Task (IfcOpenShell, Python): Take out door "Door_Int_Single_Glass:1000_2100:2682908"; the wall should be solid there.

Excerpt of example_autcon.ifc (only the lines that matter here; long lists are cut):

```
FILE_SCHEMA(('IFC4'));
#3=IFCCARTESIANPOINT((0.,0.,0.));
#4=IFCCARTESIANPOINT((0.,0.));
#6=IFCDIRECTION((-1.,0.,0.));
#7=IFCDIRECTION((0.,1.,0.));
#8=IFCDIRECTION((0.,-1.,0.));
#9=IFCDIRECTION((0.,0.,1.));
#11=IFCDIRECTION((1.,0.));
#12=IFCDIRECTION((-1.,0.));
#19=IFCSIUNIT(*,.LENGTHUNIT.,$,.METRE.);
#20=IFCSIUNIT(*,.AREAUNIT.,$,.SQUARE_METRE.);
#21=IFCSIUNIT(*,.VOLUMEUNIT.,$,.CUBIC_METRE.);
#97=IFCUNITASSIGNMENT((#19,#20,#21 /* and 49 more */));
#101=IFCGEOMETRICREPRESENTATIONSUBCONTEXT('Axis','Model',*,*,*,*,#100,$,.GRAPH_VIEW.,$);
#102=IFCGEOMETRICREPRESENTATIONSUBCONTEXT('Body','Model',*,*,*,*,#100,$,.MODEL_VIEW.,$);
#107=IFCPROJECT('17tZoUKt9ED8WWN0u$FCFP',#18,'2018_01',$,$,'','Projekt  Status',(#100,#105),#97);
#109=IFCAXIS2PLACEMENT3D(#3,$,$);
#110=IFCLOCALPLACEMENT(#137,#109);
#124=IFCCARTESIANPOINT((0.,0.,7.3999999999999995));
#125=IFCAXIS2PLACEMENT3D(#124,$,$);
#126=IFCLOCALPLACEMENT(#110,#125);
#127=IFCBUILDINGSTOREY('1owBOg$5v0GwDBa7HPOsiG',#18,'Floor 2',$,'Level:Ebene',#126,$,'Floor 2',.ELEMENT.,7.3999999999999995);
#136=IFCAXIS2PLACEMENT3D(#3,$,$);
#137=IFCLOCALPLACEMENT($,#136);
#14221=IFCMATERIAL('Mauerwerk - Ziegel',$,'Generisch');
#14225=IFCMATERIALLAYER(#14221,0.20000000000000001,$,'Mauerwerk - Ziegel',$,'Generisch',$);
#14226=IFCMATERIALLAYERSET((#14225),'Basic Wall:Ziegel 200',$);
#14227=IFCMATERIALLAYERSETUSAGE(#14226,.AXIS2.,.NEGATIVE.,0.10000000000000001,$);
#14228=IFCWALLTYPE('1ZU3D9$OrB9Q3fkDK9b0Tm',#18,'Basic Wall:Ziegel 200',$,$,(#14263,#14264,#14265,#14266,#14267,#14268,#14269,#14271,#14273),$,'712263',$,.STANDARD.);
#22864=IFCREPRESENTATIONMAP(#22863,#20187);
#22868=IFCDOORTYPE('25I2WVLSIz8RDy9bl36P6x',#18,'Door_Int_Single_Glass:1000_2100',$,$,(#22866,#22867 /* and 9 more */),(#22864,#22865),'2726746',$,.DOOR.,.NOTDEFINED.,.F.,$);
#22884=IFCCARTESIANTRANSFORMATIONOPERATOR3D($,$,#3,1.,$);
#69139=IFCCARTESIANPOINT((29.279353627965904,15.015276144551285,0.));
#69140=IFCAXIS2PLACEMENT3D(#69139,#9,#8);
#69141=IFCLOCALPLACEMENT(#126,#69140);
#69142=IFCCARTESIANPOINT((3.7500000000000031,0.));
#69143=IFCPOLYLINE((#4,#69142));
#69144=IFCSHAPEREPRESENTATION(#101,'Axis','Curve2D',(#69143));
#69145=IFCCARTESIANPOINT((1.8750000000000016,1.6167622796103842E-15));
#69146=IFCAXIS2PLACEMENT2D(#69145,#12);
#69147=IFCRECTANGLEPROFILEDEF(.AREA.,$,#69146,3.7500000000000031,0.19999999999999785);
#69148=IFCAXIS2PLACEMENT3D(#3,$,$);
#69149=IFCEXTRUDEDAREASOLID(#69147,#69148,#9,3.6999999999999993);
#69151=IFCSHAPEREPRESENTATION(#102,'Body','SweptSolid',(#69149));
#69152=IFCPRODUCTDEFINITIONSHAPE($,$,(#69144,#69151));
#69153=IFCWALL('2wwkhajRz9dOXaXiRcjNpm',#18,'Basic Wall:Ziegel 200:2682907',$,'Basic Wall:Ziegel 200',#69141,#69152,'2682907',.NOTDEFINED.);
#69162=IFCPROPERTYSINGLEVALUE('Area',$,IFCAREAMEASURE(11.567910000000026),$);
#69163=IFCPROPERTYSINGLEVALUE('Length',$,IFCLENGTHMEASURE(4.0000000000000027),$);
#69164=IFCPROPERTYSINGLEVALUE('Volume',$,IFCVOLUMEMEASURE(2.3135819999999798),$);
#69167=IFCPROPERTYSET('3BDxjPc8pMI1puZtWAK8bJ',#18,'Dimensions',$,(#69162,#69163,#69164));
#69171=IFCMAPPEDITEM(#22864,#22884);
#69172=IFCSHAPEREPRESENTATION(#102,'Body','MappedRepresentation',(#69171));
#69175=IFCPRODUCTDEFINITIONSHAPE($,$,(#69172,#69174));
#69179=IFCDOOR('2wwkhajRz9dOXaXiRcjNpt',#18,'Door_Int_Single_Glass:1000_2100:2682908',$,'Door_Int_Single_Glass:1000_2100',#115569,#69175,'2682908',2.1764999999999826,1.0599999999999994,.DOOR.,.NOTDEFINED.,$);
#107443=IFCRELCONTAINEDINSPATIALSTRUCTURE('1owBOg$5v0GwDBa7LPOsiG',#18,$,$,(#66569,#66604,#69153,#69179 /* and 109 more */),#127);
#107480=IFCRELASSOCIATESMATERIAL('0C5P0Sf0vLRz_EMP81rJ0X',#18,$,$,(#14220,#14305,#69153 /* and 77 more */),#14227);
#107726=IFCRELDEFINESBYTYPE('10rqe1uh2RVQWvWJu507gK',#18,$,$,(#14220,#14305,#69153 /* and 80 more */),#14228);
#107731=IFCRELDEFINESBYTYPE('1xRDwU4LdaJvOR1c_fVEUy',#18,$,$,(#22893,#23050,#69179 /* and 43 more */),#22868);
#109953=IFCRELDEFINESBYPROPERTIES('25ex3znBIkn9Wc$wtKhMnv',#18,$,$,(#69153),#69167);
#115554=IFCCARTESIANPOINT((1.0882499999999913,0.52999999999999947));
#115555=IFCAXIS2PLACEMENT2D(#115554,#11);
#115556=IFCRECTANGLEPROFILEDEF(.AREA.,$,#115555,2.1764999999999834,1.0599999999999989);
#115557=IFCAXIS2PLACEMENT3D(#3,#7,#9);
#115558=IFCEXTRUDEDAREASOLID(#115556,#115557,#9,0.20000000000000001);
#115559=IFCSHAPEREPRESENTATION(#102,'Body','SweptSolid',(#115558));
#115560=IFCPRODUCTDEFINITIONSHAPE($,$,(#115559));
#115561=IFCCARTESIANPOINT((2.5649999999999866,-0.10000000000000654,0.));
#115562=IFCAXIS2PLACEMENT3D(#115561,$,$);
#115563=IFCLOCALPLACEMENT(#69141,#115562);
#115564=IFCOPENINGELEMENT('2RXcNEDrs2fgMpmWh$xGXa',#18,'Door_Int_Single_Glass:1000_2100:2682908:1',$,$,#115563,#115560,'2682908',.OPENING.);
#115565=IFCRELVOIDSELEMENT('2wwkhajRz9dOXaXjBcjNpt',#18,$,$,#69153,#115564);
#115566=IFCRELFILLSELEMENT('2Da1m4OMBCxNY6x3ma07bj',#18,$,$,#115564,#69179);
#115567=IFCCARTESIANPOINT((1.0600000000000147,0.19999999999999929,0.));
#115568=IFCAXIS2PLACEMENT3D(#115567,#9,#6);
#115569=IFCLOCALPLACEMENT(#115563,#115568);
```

```python
import ifcopenshell
import ifcopenshell.api.feature
import ifcopenshell.api.pset
import ifcopenshell.api.root
import ifcopenshell.geom
import ifcopenshell.util.element
import ifcopenshell.util.shape
import ifcopenshell.util.unit

model = ifcopenshell.open("example_autcon.ifc")
area_scale = ifcopenshell.util.unit.calculate_unit_scale(model, "AREAUNIT")
volume_scale = ifcopenshell.util.unit.calculate_unit_scale(model, "VOLUMEUNIT")
settings = ifcopenshell.geom.settings()


def volume(element):
    """Net volume in cubic metres, openings subtracted."""
    shape = ifcopenshell.geom.create_shape(settings, element)
    return ifcopenshell.util.shape.get_volume(shape.geometry)


door = model.by_guid("2wwkhajRz9dOXaXiRcjNpt")
opening = door.FillsVoids[0].RelatingOpeningElement
wall = opening.VoidsElements[0].RelatingBuildingElement
before = volume(wall)

ifcopenshell.api.root.remove_product(model, product=door)
ifcopenshell.api.feature.remove_feature(model, feature=opening)

after = volume(wall)
thickness = 0.2  # wall thickness in metres

# Update the wall's stored quantities.
pset = model.by_id(ifcopenshell.util.element.get_pset(wall, "Dimensions", should_inherit=False)["id"])
ifcopenshell.api.pset.edit_pset(model, pset=pset, properties={
    "Area": model.create_entity("IfcAreaMeasure", after / thickness / area_scale),
    "Volume": model.create_entity("IfcVolumeMeasure", after / volume_scale),
})

print(f"wall volume {before:.3f} -> {after:.3f} m3")

model.write("example_autcon_updated.ifc")
```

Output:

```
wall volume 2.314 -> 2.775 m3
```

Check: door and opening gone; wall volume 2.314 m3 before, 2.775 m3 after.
